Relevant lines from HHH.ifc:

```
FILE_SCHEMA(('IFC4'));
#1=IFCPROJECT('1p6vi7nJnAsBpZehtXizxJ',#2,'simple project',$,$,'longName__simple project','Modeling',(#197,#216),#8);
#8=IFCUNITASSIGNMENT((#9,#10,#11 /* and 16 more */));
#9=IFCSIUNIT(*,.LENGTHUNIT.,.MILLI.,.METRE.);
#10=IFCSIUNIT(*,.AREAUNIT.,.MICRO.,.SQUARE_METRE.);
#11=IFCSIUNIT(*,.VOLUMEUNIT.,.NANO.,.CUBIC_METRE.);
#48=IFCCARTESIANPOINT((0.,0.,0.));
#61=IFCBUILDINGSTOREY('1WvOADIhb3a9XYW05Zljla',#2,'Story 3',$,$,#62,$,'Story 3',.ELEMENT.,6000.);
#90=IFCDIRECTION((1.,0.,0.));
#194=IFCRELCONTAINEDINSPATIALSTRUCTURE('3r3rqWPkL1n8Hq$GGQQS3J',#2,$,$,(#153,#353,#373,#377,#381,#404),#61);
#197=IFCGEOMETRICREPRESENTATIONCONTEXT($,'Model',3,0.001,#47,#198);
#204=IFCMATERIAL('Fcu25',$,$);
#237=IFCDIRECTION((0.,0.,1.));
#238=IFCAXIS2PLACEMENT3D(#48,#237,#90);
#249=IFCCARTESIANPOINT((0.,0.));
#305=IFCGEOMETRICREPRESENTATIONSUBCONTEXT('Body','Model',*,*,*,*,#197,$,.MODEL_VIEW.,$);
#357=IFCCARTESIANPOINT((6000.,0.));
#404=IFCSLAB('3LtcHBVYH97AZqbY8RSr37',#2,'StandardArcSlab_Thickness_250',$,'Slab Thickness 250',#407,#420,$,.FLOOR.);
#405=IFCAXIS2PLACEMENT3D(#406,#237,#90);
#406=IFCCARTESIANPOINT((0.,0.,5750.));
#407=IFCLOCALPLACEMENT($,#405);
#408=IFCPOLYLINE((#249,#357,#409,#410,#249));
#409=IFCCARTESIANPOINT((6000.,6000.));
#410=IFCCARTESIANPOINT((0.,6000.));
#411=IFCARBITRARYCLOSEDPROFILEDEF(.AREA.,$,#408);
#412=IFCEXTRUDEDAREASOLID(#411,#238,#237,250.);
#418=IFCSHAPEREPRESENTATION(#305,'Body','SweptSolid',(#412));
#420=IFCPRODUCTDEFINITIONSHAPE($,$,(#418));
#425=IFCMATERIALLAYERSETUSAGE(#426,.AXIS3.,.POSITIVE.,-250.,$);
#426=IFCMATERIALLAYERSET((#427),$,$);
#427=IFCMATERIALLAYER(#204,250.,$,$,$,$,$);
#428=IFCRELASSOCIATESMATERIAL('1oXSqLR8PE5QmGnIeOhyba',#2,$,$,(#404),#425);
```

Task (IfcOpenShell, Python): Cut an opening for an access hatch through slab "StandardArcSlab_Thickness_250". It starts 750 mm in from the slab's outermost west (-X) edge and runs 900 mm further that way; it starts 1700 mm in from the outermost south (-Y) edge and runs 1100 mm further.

```python
import numpy as np
import ifcopenshell
import ifcopenshell.api.feature
import ifcopenshell.api.geometry
import ifcopenshell.api.root
import ifcopenshell.geom
import ifcopenshell.util.placement
import ifcopenshell.util.representation
import ifcopenshell.util.shape
import ifcopenshell.util.unit

model = ifcopenshell.open("HHH.ifc")
unit_scale = ifcopenshell.util.unit.calculate_unit_scale(model)
settings = ifcopenshell.geom.settings()


def volume(element):
    """Net volume in cubic metres, openings subtracted."""
    shape = ifcopenshell.geom.create_shape(settings, element)
    return ifcopenshell.util.shape.get_volume(shape.geometry)


slab = model.by_guid("3LtcHBVYH97AZqbY8RSr37")
before = volume(slab)

# Extent in the slab's own axes, in metres. The edges named are its -X and -Y sides.
slab_shape = ifcopenshell.geom.create_shape(settings, slab)
vertices = ifcopenshell.util.shape.get_vertices(slab_shape.geometry)
x_min, y_min, bottom = vertices.min(axis=0)
top = vertices[:, 2].max()

opening = ifcopenshell.api.root.create_entity(model, ifc_class="IfcOpeningElement", name="Access hatch opening", predefined_type="OPENING")
context = ifcopenshell.util.representation.get_context(model, "Model", "Body", "MODEL_VIEW")
width, depth = 0.9, 1.1
outline = [(0.0, 0.0), (width, 0.0), (width, depth), (0.0, depth), (0.0, 0.0)]
# Overshoot both faces by 50 mm so the cut is clean.
shape = ifcopenshell.api.geometry.add_slab_representation(
    model, context=context, depth=top - bottom + 0.1, polyline=outline
)
ifcopenshell.api.geometry.assign_representation(model, product=opening, representation=shape)

matrix = ifcopenshell.util.placement.get_local_placement(slab.ObjectPlacement)
matrix[:, 3] = matrix @ np.append(np.array([x_min + 0.75, y_min + 1.7, bottom - 0.05]) / unit_scale, 1.0)
ifcopenshell.api.geometry.edit_object_placement(model, product=opening, matrix=matrix, is_si=False)
ifcopenshell.api.feature.add_feature(model, feature=opening, element=slab)

after = volume(slab)

print(f"slab volume {before:.3f} -> {after:.3f} m3")

model.write("HHH_updated.ifc")
```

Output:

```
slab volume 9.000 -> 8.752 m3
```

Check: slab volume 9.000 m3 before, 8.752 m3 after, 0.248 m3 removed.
